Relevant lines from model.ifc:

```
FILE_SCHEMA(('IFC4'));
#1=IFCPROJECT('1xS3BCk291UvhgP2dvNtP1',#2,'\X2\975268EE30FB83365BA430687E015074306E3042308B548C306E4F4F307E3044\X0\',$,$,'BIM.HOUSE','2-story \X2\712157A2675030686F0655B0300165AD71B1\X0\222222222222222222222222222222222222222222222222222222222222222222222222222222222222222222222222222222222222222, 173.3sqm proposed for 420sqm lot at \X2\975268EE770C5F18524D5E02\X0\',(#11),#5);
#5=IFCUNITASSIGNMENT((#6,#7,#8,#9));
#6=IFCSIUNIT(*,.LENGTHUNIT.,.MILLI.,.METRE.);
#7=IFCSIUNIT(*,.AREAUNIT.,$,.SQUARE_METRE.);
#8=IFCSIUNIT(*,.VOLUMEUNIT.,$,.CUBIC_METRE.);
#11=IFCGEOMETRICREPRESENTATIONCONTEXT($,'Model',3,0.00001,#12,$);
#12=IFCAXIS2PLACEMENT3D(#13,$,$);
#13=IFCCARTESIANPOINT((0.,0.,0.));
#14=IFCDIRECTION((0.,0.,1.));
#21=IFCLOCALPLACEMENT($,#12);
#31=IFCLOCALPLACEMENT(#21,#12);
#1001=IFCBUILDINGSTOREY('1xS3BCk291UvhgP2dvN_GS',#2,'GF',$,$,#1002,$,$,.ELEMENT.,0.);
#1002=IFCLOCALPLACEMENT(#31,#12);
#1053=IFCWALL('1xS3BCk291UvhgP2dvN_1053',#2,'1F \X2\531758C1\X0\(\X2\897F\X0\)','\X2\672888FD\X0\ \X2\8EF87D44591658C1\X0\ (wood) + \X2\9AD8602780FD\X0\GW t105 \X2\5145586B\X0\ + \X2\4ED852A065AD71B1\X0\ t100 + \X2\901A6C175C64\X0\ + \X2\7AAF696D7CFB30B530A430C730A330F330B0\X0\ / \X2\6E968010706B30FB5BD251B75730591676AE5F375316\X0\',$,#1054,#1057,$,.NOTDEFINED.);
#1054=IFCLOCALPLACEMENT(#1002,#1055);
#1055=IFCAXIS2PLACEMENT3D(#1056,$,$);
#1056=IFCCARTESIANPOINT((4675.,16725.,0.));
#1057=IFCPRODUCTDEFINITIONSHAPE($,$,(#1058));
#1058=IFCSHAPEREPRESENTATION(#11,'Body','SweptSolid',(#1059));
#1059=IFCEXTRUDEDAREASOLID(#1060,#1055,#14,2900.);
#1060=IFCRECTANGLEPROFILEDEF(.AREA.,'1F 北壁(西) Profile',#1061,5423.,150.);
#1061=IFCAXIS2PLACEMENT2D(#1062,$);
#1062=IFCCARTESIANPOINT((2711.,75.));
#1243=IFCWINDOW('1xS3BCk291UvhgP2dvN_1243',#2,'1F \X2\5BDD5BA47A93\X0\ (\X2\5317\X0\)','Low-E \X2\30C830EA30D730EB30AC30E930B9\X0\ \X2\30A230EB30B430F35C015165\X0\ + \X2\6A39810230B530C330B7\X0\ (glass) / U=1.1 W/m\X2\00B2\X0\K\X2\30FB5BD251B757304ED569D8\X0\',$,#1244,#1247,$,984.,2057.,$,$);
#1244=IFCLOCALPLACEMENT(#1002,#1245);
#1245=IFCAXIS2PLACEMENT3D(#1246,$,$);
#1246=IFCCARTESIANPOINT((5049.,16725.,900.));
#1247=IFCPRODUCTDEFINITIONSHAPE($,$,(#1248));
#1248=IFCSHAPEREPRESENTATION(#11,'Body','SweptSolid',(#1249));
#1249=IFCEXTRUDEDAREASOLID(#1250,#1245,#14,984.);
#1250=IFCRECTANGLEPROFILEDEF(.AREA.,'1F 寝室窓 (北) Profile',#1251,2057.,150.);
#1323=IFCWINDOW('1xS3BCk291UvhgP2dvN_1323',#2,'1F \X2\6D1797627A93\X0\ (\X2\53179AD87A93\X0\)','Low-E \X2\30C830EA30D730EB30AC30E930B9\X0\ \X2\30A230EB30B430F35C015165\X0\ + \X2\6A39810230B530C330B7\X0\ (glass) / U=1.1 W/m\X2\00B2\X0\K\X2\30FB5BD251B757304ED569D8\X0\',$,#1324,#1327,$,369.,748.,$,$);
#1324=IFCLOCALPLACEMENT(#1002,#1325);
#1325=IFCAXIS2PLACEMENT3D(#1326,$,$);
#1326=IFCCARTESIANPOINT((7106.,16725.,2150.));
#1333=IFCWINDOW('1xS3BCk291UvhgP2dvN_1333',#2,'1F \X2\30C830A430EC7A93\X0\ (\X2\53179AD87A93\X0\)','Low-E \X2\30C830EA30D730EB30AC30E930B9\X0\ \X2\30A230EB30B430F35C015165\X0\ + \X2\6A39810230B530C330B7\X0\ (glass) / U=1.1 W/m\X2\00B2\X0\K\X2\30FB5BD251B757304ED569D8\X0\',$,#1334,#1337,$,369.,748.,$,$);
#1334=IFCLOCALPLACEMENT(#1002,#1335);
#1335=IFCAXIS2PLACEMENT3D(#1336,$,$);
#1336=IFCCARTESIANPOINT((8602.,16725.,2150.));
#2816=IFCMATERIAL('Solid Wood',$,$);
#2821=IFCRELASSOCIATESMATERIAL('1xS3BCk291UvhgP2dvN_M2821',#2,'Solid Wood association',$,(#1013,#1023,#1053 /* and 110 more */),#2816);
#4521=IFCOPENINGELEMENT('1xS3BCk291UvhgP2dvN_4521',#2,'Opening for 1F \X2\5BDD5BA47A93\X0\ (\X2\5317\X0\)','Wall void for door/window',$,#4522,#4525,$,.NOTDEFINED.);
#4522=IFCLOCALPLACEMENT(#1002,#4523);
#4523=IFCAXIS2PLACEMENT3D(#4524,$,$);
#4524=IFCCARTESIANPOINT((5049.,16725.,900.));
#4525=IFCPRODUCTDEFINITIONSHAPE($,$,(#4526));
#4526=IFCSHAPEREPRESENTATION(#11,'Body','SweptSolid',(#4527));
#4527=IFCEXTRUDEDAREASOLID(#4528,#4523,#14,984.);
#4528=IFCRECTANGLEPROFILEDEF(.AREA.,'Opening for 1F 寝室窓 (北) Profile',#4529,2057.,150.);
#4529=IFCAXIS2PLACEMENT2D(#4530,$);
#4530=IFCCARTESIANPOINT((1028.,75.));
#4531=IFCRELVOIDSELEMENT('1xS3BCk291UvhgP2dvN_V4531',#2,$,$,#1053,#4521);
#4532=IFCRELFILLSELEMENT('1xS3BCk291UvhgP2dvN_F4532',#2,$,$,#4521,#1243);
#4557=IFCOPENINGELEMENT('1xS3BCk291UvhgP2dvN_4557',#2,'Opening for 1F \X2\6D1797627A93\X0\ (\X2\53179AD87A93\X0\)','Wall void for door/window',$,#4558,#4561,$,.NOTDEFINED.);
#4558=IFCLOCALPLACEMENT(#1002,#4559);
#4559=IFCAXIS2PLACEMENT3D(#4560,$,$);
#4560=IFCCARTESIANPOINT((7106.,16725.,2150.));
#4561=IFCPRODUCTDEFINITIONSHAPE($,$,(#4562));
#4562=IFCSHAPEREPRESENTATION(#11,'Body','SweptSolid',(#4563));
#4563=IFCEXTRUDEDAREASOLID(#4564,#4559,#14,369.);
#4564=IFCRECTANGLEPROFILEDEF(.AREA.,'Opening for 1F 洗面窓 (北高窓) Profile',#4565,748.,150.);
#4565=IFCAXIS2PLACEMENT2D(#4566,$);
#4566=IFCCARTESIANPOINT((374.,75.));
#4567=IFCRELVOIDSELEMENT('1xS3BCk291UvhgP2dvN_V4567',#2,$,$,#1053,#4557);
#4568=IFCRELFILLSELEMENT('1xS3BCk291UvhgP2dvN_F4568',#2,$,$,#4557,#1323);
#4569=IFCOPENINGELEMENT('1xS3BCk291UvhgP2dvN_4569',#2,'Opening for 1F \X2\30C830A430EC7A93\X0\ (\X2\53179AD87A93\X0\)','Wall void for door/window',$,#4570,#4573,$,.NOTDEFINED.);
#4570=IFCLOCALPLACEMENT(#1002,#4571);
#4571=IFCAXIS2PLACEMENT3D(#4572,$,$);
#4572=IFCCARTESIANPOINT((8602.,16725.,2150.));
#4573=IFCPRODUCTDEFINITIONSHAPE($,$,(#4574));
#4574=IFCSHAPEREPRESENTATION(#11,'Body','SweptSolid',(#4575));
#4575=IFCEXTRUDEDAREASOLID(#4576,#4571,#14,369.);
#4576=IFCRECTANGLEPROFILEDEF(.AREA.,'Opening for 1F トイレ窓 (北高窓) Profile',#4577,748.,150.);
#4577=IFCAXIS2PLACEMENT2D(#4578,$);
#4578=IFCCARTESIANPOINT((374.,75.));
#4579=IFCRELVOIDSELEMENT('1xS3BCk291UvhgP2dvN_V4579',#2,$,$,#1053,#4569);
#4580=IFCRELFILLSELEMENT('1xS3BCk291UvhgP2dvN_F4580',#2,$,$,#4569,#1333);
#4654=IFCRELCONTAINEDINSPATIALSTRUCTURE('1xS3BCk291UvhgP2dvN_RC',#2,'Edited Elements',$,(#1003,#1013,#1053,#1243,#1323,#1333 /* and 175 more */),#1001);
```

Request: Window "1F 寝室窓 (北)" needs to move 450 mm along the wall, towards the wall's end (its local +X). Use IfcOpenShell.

```python
import ifcopenshell
import ifcopenshell.api.geometry
import ifcopenshell.util.placement

model = ifcopenshell.open("model.ifc")

window = model.by_guid("1xS3BCk291UvhgP2dvN_1243")
opening = window.FillsVoids[0].RelatingOpeningElement
wall = opening.VoidsElements[0].RelatingBuildingElement

wall_matrix = ifcopenshell.util.placement.get_local_placement(wall.ObjectPlacement)
shift = wall_matrix[:3, 0] * 450.0
before = ifcopenshell.util.placement.get_local_placement(window.ObjectPlacement)[:3, 3].copy()

# The window is not placed relative to its opening, so move both.
for product in (opening, window):
    matrix = ifcopenshell.util.placement.get_local_placement(product.ObjectPlacement)
    matrix[:3, 3] += shift
    ifcopenshell.api.geometry.edit_object_placement(model, product=product, matrix=matrix, is_si=False)

after = ifcopenshell.util.placement.get_local_placement(window.ObjectPlacement)[:3, 3]
print("window moved by", (after - before).round(3) + 0.0)

model.write("model_rev.ifc")
```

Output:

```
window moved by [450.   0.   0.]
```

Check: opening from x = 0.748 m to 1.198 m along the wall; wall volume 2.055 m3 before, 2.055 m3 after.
